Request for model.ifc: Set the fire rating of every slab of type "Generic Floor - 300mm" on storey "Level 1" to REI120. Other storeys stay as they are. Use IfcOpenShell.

First a look at what the model holds.

```python
import ifcopenshell
import ifcopenshell.util.element

model = ifcopenshell.open("model.ifc")
print(model.schema)
storey = next(s for s in model.by_type("IfcBuildingStorey") if s.Name == "Level 1")
slabs = [e for e in ifcopenshell.util.element.get_decomposition(storey) if e.is_a("IfcSlab")]
seen = {}
for e in slabs:
    element_type = ifcopenshell.util.element.get_type(e)
    key = (element_type.Name if element_type != e and element_type else None, ifcopenshell.util.element.get_pset(e, "Pset_SlabCommon", "FireRating"))
    seen[key] = seen.get(key, 0) + 1
for (name, value), count in sorted(seen.items(), key=str):
    print(count, "x", name, "|", value)
```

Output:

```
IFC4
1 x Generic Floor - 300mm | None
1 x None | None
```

```python
import ifcopenshell
import ifcopenshell.api.pset
import ifcopenshell.util.element

model = ifcopenshell.open("model.ifc")

storey = next(s for s in model.by_type("IfcBuildingStorey") if s.Name == "Level 1")
slabs = [e for e in ifcopenshell.util.element.get_decomposition(storey) if e.is_a("IfcSlab")]

count = 0
for e in slabs:
    element_type = ifcopenshell.util.element.get_type(e)
    if element_type in (None, e) or element_type.Name != "Generic Floor - 300mm":
        continue
    # add_pset returns the element's existing set when there is one.
    pset = ifcopenshell.api.pset.add_pset(model, product=e, name="Pset_SlabCommon")
    ifcopenshell.api.pset.edit_pset(model, pset=pset, properties={"FireRating": "REI120"})
    count += 1

print(count, "slabs updated")

model.write("model_rev.ifc")
```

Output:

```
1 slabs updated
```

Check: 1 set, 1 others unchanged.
